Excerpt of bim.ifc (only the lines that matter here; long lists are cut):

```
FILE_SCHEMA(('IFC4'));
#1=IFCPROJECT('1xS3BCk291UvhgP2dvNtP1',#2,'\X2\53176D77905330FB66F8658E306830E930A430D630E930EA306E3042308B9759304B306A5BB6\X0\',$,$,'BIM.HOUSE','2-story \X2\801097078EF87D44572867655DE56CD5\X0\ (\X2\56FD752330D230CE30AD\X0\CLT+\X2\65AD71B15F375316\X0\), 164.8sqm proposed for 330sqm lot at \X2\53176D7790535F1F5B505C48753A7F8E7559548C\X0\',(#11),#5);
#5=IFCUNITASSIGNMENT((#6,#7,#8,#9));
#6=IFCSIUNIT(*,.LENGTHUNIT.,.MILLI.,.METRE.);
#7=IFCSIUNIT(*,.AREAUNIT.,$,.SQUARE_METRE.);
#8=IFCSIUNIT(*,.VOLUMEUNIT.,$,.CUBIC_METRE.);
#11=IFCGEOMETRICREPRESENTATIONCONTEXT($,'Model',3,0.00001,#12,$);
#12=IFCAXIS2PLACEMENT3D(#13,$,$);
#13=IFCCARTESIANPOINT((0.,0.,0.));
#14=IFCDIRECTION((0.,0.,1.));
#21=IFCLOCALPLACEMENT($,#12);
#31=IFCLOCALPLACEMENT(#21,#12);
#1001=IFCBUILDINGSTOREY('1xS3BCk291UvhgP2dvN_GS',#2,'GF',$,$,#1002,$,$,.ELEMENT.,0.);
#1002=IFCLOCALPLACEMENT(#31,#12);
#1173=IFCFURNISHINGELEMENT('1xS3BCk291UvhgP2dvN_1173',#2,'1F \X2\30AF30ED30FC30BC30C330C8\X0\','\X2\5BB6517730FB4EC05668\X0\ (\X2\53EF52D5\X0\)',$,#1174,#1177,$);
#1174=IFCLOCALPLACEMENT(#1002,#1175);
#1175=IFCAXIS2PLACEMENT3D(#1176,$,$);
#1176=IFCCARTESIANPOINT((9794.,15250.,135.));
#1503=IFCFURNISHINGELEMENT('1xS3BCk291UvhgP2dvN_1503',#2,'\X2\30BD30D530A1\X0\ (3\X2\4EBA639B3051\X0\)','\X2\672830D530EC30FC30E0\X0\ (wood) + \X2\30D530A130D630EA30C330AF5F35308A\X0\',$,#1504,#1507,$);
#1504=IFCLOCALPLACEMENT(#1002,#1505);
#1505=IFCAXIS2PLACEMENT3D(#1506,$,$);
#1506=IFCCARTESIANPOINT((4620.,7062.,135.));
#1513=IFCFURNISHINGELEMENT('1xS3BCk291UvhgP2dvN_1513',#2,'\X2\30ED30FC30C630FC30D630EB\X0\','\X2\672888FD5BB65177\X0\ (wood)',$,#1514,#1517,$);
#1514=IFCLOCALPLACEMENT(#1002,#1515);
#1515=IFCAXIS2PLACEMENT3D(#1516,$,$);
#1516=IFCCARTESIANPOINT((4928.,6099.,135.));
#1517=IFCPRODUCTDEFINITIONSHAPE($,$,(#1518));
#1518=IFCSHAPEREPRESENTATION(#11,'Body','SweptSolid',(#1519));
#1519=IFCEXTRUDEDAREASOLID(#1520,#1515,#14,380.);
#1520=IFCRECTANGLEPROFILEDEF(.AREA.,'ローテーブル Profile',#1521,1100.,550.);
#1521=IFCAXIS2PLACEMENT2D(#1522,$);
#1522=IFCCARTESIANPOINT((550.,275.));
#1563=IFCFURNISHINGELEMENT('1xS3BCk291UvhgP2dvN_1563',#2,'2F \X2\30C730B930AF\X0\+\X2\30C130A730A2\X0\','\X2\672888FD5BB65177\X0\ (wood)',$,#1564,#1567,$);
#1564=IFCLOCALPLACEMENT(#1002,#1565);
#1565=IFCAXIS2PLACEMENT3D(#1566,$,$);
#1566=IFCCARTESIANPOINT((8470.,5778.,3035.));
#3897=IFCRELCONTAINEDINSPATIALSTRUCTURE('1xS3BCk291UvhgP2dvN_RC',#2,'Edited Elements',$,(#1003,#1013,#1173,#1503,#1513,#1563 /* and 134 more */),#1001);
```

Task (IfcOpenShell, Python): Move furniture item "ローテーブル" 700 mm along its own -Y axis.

```python
import ifcopenshell
import ifcopenshell.api.geometry
import ifcopenshell.util.placement

model = ifcopenshell.open("bim.ifc")

item = model.by_guid("1xS3BCk291UvhgP2dvN_1513")
matrix = ifcopenshell.util.placement.get_local_placement(item.ObjectPlacement)
matrix[:3, 3] -= matrix[:3, 1] * 700.0
ifcopenshell.api.geometry.edit_object_placement(model, product=item, matrix=matrix, is_si=False)

print(ifcopenshell.util.placement.get_local_placement(item.ObjectPlacement).round(3) + 0.0)

model.write("bim_updated.ifc")
```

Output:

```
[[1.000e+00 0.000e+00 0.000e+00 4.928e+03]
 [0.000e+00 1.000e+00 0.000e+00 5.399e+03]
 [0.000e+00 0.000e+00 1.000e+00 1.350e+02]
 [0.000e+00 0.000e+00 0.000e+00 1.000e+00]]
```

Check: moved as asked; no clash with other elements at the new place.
